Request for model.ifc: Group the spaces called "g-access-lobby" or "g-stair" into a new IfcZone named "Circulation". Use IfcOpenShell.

First a look at what the model holds.

```python
import ifcopenshell

model = ifcopenshell.open("model.ifc")
print(model.schema)
seen = {}
for space in model.by_type("IfcSpace"):
    seen[space.LongName] = seen.get(space.LongName, 0) + 1
for name, count in sorted(seen.items(), key=str):
    print(count, "x", name)
print("zones:", [z.Name for z in model.by_type("IfcZone")][:20])
```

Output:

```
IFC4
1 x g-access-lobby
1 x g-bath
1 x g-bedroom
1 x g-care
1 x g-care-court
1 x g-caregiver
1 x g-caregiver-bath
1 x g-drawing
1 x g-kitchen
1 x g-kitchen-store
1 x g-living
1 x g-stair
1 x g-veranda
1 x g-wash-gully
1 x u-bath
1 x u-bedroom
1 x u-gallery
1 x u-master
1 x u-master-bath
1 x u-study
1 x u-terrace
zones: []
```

```python
import ifcopenshell
import ifcopenshell.api.group
import ifcopenshell.api.root

model = ifcopenshell.open("model.ifc")

names = {"g-access-lobby", "g-stair"}
spaces = [s for s in model.by_type("IfcSpace") if s.LongName in names]

zone = ifcopenshell.api.root.create_entity(model, ifc_class="IfcZone", name="Circulation")
ifcopenshell.api.group.assign_group(model, products=spaces, group=zone)
print(len(spaces), "spaces in", zone.Name)

model.write("model_edited.ifc")
```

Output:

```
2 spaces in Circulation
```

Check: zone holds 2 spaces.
